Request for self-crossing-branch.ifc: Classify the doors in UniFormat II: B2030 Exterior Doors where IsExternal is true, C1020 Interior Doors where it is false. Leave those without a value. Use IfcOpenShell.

First a look at what the model holds.

```python
import ifcopenshell
import ifcopenshell.util.element

model = ifcopenshell.open("self-crossing-branch.ifc")
print(model.schema)
print("classifications:", [c.Name for c in model.by_type("IfcClassification")])
values = [ifcopenshell.util.element.get_pset(e, "Pset_DoorCommon", "IsExternal") for e in model.by_type("IfcDoor")]
for value in (True, False, None):
    print("IsExternal", value, values.count(value))
```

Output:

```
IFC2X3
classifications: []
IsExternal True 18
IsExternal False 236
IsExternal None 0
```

```python
import ifcopenshell
import ifcopenshell.api.classification
import ifcopenshell.util.element

model = ifcopenshell.open("self-crossing-branch.ifc")

# IFC2X3 requires Source and Edition and has no link from the project to the system.
system = model.create_entity("IfcClassification", Source="ASTM", Edition="E1557", Name="UniFormat II")

doors = model.by_type("IfcDoor")
external = {e: ifcopenshell.util.element.get_pset(e, "Pset_DoorCommon", "IsExternal") for e in doors}
for flag, code, name in ((True, "B2030", "Exterior Doors"), (False, "C1020", "Interior Doors")):
    products = [e for e in doors if external[e] is flag]
    ifcopenshell.api.classification.add_reference(
        model, products=products, classification=system, identification=code, name=name
    )
    print(code, len(products))

model.write("self-crossing-branch_edited.ifc")
```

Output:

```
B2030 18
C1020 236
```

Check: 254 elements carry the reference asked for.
